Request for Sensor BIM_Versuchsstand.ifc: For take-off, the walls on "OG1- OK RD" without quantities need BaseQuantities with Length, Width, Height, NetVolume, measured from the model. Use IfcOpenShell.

First a look at what the model holds.

```python
import ifcopenshell
import ifcopenshell.util.element
import ifcopenshell.util.unit

model = ifcopenshell.open("Sensor BIM_Versuchsstand.ifc")
print(model.schema)
for unit_type in ("LENGTHUNIT", "AREAUNIT", "VOLUMEUNIT"):
    print(unit_type, ifcopenshell.util.unit.calculate_unit_scale(model, unit_type))
storey = next(s for s in model.by_type("IfcBuildingStorey") if s.Name == "OG1- OK RD")
walls = [e for e in ifcopenshell.util.element.get_decomposition(storey) if e.is_a("IfcWall")]
for e in sorted(walls, key=lambda e: e.id()):
    print(e.id(), e.is_a(), e.Name, list(ifcopenshell.util.element.get_psets(e, qtos_only=True)), sep=" | ")
```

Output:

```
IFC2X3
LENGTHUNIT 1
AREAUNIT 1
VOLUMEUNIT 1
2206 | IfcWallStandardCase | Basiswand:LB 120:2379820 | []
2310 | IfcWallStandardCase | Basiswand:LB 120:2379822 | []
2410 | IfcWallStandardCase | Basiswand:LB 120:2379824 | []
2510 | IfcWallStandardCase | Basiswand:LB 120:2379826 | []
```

```python
import ifcopenshell
import ifcopenshell.api.pset
import ifcopenshell.geom
import ifcopenshell.util.element
import ifcopenshell.util.shape
import ifcopenshell.util.unit

model = ifcopenshell.open("Sensor BIM_Versuchsstand.ifc")
unit_scale = ifcopenshell.util.unit.calculate_unit_scale(model)
volume_scale = ifcopenshell.util.unit.calculate_unit_scale(model, "VOLUMEUNIT")
settings = ifcopenshell.geom.settings()

storey = next(s for s in model.by_type("IfcBuildingStorey") if s.Name == "OG1- OK RD")
walls = [e for e in ifcopenshell.util.element.get_decomposition(storey) if e.is_a("IfcWall")]

for e in sorted(walls, key=lambda e: e.id()):
    if ifcopenshell.util.element.get_psets(e, qtos_only=True, should_inherit=False):
        continue
    # Geometry comes back in metres, in the element's own axes.
    shape = ifcopenshell.geom.create_shape(settings, e)
    values = {
        "Length": ifcopenshell.util.shape.get_x(shape.geometry) / unit_scale,
        "Width": ifcopenshell.util.shape.get_y(shape.geometry) / unit_scale,
        "Height": ifcopenshell.util.shape.get_z(shape.geometry) / unit_scale,
        "NetVolume": ifcopenshell.util.shape.get_volume(shape.geometry) / volume_scale,
    }
    qto = ifcopenshell.api.pset.add_qto(model, product=e, name="BaseQuantities")
    ifcopenshell.api.pset.edit_qto(model, qto=qto, properties=values)
    print(e.id(), {k: round(v, 3) for k, v in values.items()})

model.write("Sensor BIM_Versuchsstand_v2.ifc")
```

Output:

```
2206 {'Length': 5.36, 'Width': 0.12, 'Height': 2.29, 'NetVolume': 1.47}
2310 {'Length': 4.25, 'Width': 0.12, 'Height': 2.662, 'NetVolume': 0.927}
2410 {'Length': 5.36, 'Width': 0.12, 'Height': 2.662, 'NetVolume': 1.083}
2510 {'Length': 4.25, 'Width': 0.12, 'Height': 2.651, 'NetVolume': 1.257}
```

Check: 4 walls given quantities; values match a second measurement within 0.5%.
